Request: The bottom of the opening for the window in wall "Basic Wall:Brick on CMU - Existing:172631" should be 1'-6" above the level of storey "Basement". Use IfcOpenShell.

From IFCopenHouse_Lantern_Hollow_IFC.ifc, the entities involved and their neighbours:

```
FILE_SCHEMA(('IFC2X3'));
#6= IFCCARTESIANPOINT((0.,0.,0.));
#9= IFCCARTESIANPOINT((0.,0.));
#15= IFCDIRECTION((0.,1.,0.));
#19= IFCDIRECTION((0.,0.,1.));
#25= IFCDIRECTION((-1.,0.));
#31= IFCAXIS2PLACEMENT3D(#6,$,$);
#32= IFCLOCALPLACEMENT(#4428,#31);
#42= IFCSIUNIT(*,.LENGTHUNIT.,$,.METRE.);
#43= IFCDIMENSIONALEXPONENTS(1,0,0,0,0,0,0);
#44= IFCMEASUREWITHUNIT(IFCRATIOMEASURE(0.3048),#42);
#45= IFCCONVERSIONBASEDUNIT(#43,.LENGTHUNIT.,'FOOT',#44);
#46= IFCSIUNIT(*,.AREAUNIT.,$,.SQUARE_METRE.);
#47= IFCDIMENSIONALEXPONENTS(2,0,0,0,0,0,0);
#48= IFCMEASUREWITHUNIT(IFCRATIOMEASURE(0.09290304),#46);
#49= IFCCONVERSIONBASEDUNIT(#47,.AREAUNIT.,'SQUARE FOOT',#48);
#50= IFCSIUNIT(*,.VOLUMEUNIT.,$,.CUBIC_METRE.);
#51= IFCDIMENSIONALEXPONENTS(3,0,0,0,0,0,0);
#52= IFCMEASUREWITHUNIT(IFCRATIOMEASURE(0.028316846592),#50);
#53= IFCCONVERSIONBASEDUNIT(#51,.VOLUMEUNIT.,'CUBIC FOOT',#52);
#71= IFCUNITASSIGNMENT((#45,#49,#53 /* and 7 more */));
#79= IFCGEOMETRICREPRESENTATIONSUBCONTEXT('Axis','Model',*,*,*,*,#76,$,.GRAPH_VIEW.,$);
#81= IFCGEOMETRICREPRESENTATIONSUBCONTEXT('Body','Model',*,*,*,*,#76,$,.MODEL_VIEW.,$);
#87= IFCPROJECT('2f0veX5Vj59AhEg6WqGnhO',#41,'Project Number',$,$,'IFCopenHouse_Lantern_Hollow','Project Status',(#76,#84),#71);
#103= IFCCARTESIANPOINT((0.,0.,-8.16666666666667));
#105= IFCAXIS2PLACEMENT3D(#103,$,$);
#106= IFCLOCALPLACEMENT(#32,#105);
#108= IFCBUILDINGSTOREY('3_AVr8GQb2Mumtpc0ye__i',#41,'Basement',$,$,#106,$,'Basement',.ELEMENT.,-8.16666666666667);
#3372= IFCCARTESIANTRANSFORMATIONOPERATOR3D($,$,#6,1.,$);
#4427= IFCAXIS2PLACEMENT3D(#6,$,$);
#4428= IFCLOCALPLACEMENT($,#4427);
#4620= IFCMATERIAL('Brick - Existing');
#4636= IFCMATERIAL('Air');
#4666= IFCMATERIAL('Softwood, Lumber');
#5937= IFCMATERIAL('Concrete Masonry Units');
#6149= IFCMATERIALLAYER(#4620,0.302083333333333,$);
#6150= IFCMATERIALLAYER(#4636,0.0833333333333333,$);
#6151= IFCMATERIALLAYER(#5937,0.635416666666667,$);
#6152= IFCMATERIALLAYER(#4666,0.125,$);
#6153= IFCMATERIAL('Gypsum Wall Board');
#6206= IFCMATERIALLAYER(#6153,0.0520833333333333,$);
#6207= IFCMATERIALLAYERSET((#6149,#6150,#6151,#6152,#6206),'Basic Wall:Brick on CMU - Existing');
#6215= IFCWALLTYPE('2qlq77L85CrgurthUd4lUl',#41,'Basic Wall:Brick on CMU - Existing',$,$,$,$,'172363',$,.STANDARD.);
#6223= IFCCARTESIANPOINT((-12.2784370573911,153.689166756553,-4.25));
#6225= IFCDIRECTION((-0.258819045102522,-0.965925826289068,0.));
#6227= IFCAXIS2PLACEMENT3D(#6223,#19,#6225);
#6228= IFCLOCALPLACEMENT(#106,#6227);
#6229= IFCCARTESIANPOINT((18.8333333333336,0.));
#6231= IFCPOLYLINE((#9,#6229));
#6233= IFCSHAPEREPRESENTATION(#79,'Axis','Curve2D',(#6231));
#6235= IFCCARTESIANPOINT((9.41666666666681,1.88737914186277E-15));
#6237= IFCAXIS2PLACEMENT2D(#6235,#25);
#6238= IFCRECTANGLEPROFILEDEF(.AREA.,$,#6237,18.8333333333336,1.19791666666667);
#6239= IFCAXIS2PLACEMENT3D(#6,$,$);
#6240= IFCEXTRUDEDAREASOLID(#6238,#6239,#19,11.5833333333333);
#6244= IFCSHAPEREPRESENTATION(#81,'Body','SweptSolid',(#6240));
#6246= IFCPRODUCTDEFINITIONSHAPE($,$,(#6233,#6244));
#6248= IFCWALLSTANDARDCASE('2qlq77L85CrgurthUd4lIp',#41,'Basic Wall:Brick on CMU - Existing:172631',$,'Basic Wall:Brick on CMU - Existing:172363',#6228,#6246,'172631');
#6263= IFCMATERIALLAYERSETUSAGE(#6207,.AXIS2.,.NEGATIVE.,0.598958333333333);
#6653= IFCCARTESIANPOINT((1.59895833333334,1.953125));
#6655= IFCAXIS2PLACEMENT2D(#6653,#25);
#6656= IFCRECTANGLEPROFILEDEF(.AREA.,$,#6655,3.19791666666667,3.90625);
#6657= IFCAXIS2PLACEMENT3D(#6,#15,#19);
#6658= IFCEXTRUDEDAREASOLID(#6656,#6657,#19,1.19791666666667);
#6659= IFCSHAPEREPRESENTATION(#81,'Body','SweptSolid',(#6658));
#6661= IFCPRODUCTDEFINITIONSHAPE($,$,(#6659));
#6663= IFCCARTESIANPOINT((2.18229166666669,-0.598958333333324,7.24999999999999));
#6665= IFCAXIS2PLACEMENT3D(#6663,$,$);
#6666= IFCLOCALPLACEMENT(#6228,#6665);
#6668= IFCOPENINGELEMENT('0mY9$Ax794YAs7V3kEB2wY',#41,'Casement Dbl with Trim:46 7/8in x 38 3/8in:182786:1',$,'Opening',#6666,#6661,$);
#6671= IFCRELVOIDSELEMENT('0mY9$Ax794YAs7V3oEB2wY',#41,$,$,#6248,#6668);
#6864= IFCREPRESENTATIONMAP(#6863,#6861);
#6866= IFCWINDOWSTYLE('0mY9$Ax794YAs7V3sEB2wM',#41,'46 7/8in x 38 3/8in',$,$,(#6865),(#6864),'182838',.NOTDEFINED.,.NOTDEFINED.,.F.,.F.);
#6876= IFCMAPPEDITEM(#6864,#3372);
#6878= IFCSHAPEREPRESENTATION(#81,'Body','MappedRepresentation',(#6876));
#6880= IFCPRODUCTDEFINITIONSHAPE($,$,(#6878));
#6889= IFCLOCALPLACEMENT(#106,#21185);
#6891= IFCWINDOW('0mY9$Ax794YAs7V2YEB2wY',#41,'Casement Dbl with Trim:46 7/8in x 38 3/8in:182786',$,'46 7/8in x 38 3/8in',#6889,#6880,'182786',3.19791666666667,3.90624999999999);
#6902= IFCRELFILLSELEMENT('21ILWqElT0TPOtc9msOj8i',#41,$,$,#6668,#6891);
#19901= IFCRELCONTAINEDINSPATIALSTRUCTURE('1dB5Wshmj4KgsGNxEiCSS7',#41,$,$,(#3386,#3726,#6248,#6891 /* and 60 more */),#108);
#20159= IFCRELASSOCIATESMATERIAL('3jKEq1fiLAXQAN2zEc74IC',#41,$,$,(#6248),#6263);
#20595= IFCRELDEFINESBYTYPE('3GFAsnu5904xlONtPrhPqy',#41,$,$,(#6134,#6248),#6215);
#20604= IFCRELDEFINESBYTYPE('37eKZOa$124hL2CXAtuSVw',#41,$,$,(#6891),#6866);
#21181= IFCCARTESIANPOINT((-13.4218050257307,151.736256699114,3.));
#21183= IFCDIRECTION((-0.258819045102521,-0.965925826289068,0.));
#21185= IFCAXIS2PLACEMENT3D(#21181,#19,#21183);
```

```python
import numpy as np
import ifcopenshell
import ifcopenshell.api.geometry
import ifcopenshell.geom
import ifcopenshell.util.element
import ifcopenshell.util.placement
import ifcopenshell.util.shape
import ifcopenshell.util.unit

model = ifcopenshell.open("IFCopenHouse_Lantern_Hollow_IFC.ifc")
unit_scale = ifcopenshell.util.unit.calculate_unit_scale(model)

window = model.by_guid("0mY9$Ax794YAs7V2YEB2wY")
opening = window.FillsVoids[0].RelatingOpeningElement
storey = ifcopenshell.util.element.get_container(window, ifc_class="IfcBuildingStorey")
level = ifcopenshell.util.placement.get_local_placement(storey.ObjectPlacement)[2, 3]

# The opening's origin need not be at the sill, so measure its lowest point.
shape = ifcopenshell.geom.create_shape(ifcopenshell.geom.settings(), opening)
bottom = ifcopenshell.util.shape.get_shape_bottom_elevation(shape, shape.geometry) / unit_scale
dz = level + 18 * 0.0254 / unit_scale - bottom

shift = np.array([0.0, 0.0, dz])
# The window is not placed relative to its opening, so move both.
for product in (opening, window):
    matrix = ifcopenshell.util.placement.get_local_placement(product.ObjectPlacement)
    matrix[:3, 3] += shift
    ifcopenshell.api.geometry.edit_object_placement(model, product=product, matrix=matrix, is_si=False)

print(f"moved by {dz * unit_scale:+.3f} m")

model.write("IFCopenHouse_Lantern_Hollow_IFC_rev.ifc")
```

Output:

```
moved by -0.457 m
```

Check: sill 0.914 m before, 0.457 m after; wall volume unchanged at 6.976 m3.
